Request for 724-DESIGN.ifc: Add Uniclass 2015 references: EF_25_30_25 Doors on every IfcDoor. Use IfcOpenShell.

First a look at what the model holds.

```python
import ifcopenshell

model = ifcopenshell.open("724-DESIGN.ifc")
print(model.schema)
print("classifications:", [c.Name for c in model.by_type("IfcClassification")])
for ifc_class in ("IfcDoor", "IfcRoof", "IfcStair", "IfcWall", "IfcWindow"):
    print(ifc_class, len(model.by_type(ifc_class)))
```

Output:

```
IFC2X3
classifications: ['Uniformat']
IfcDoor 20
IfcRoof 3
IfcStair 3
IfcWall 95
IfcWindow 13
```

```python
import ifcopenshell
import ifcopenshell.api.classification

model = ifcopenshell.open("724-DESIGN.ifc")

# IFC2X3 requires Source and Edition and has no link from the project to the system.
system = model.create_entity("IfcClassification", Source="NBS", Edition="2015", Name="Uniclass 2015")

codes = {
    "IfcDoor": ("EF_25_30_25", "Doors"),
}
for ifc_class, (code, name) in codes.items():
    products = model.by_type(ifc_class)
    ifcopenshell.api.classification.add_reference(
        model, products=products, classification=system, identification=code, name=name
    )
    print(code, len(products))

model.write("724-DESIGN-out.ifc")
```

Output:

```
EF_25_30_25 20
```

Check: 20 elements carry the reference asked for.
